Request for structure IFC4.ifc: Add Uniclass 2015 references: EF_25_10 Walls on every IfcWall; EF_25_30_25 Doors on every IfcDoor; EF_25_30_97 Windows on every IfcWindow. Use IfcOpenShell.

First a look at what the model holds.

```python
import ifcopenshell

model = ifcopenshell.open("structure IFC4.ifc")
print(model.schema)
print("classifications:", [c.Name for c in model.by_type("IfcClassification")])
for ifc_class in ("IfcDoor", "IfcRoof", "IfcStair", "IfcWall", "IfcWindow"):
    print(ifc_class, len(model.by_type(ifc_class)))
```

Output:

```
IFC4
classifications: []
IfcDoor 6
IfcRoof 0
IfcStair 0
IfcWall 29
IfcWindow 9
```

```python
import ifcopenshell
import ifcopenshell.api.classification

model = ifcopenshell.open("structure IFC4.ifc")

system = ifcopenshell.api.classification.add_classification(model, classification="Uniclass 2015")

codes = {
    "IfcWall": ("EF_25_10", "Walls"),
    "IfcDoor": ("EF_25_30_25", "Doors"),
    "IfcWindow": ("EF_25_30_97", "Windows"),
}
for ifc_class, (code, name) in codes.items():
    products = model.by_type(ifc_class)
    ifcopenshell.api.classification.add_reference(
        model, products=products, classification=system, identification=code, name=name
    )
    print(code, len(products))

model.write("structure IFC4-out.ifc")
```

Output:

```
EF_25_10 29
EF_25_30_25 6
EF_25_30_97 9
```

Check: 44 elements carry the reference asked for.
